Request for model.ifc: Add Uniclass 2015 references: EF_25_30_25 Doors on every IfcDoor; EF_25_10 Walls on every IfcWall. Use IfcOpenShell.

First a look at what the model holds.

```python
import ifcopenshell

model = ifcopenshell.open("model.ifc")
print(model.schema)
print("classifications:", [c.Name for c in model.by_type("IfcClassification")])
for ifc_class in ("IfcDoor", "IfcRoof", "IfcStair", "IfcWall", "IfcWindow"):
    print(ifc_class, len(model.by_type(ifc_class)))
```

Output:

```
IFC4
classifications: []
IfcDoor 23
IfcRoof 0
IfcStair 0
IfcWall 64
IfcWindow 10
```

```python
import ifcopenshell
import ifcopenshell.api.classification

model = ifcopenshell.open("model.ifc")

system = ifcopenshell.api.classification.add_classification(model, classification="Uniclass 2015")

codes = {
    "IfcDoor": ("EF_25_30_25", "Doors"),
    "IfcWall": ("EF_25_10", "Walls"),
}
for ifc_class, (code, name) in codes.items():
    products = model.by_type(ifc_class)
    ifcopenshell.api.classification.add_reference(
        model, products=products, classification=system, identification=code, name=name
    )
    print(code, len(products))

model.write("model_rev.ifc")
```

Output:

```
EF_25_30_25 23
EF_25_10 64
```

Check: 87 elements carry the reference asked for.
